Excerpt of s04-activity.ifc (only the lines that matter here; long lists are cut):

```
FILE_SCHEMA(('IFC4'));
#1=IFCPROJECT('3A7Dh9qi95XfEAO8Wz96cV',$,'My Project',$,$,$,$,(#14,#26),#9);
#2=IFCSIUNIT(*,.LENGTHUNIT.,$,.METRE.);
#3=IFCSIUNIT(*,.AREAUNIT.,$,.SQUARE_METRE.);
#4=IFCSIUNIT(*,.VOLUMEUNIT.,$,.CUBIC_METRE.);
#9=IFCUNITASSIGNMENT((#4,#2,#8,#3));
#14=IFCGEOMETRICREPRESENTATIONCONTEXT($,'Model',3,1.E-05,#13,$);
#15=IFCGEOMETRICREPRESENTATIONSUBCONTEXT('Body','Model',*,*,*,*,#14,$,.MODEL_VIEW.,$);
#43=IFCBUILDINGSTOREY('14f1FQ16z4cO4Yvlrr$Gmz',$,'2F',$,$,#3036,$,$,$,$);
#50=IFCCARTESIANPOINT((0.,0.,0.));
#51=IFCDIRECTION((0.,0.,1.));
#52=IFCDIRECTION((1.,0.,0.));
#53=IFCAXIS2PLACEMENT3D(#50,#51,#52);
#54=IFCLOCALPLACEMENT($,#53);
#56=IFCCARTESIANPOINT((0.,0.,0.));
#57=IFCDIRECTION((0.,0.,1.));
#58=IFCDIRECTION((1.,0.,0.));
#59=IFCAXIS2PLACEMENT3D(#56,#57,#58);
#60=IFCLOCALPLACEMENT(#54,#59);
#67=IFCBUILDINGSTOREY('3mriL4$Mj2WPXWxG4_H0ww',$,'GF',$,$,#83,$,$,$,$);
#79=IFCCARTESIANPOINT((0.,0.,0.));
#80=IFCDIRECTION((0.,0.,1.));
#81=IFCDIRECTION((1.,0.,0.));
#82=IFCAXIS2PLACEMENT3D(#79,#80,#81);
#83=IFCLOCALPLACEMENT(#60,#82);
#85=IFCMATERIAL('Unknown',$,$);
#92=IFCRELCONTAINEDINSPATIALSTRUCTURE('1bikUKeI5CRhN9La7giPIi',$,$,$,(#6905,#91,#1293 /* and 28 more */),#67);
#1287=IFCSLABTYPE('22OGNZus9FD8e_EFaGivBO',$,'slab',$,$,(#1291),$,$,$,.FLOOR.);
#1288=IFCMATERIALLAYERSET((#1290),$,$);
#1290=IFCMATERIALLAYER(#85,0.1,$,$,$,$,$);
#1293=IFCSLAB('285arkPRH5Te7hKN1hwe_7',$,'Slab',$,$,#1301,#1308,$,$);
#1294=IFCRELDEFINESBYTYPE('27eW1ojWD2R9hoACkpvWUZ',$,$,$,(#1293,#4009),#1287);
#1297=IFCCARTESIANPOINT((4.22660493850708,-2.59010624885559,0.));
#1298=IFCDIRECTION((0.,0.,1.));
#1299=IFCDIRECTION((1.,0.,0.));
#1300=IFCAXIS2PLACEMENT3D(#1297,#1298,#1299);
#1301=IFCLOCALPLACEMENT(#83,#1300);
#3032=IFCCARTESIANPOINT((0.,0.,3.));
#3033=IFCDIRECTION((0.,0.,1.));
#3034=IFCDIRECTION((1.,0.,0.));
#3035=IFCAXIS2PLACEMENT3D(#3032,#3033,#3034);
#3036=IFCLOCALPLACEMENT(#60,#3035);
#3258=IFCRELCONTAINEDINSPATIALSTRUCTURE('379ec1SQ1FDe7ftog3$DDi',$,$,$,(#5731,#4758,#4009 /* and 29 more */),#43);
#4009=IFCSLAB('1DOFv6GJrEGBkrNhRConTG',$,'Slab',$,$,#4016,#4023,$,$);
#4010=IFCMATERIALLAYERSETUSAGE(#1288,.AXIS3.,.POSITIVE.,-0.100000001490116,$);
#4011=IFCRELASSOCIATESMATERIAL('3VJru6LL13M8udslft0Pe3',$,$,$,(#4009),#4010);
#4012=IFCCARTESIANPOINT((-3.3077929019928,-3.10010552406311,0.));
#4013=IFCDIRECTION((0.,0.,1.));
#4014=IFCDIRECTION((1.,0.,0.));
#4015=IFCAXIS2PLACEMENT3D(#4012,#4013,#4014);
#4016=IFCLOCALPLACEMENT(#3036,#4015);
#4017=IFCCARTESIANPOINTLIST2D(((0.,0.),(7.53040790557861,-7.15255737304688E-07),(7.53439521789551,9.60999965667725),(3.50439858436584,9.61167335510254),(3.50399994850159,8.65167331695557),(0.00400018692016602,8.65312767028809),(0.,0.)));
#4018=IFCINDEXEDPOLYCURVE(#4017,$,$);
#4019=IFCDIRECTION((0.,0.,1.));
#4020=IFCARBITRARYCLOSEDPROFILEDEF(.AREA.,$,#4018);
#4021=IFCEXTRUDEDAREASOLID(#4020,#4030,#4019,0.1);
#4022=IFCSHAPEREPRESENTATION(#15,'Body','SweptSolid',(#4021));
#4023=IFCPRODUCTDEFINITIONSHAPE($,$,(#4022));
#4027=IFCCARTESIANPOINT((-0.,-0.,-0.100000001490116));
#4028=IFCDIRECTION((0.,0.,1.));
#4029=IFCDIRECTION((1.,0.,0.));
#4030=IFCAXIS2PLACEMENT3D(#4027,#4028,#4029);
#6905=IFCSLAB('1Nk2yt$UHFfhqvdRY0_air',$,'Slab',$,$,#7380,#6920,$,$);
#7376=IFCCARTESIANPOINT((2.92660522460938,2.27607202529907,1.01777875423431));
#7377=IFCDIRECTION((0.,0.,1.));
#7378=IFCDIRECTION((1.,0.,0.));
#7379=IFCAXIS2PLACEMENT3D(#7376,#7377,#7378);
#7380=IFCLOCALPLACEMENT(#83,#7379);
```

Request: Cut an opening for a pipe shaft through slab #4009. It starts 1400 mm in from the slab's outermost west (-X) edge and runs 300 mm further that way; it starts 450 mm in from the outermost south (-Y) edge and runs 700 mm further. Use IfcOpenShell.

```python
import numpy as np
import ifcopenshell
import ifcopenshell.api.feature
import ifcopenshell.api.geometry
import ifcopenshell.api.root
import ifcopenshell.geom
import ifcopenshell.util.placement
import ifcopenshell.util.representation
import ifcopenshell.util.shape
import ifcopenshell.util.unit

model = ifcopenshell.open("s04-activity.ifc")
unit_scale = ifcopenshell.util.unit.calculate_unit_scale(model)
settings = ifcopenshell.geom.settings()


def volume(element):
    """Net volume in cubic metres, openings subtracted."""
    shape = ifcopenshell.geom.create_shape(settings, element)
    return ifcopenshell.util.shape.get_volume(shape.geometry)


slab = model.by_id(4009)
before = volume(slab)

# Extent in the slab's own axes, in metres. The edges named are its -X and -Y sides.
slab_shape = ifcopenshell.geom.create_shape(settings, slab)
vertices = ifcopenshell.util.shape.get_vertices(slab_shape.geometry)
x_min, y_min, bottom = vertices.min(axis=0)
top = vertices[:, 2].max()

opening = ifcopenshell.api.root.create_entity(model, ifc_class="IfcOpeningElement", name="Pipe shaft opening", predefined_type="OPENING")
context = ifcopenshell.util.representation.get_context(model, "Model", "Body", "MODEL_VIEW")
width, depth = 0.3, 0.7
outline = [(0.0, 0.0), (width, 0.0), (width, depth), (0.0, depth), (0.0, 0.0)]
# Overshoot both faces by 50 mm so the cut is clean.
shape = ifcopenshell.api.geometry.add_slab_representation(
    model, context=context, depth=top - bottom + 0.1, polyline=outline
)
ifcopenshell.api.geometry.assign_representation(model, product=opening, representation=shape)

matrix = ifcopenshell.util.placement.get_local_placement(slab.ObjectPlacement)
matrix[:, 3] = matrix @ np.append(np.array([x_min + 1.4, y_min + 0.45, bottom - 0.05]) / unit_scale, 1.0)
ifcopenshell.api.geometry.edit_object_placement(model, product=opening, matrix=matrix, is_si=False)
ifcopenshell.api.feature.add_feature(model, feature=opening, element=slab)

after = volume(slab)

print(f"slab volume {before:.3f} -> {after:.3f} m3")

model.write("s04-activity_updated.ifc")
```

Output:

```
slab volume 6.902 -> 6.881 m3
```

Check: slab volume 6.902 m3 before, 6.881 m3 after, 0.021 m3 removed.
